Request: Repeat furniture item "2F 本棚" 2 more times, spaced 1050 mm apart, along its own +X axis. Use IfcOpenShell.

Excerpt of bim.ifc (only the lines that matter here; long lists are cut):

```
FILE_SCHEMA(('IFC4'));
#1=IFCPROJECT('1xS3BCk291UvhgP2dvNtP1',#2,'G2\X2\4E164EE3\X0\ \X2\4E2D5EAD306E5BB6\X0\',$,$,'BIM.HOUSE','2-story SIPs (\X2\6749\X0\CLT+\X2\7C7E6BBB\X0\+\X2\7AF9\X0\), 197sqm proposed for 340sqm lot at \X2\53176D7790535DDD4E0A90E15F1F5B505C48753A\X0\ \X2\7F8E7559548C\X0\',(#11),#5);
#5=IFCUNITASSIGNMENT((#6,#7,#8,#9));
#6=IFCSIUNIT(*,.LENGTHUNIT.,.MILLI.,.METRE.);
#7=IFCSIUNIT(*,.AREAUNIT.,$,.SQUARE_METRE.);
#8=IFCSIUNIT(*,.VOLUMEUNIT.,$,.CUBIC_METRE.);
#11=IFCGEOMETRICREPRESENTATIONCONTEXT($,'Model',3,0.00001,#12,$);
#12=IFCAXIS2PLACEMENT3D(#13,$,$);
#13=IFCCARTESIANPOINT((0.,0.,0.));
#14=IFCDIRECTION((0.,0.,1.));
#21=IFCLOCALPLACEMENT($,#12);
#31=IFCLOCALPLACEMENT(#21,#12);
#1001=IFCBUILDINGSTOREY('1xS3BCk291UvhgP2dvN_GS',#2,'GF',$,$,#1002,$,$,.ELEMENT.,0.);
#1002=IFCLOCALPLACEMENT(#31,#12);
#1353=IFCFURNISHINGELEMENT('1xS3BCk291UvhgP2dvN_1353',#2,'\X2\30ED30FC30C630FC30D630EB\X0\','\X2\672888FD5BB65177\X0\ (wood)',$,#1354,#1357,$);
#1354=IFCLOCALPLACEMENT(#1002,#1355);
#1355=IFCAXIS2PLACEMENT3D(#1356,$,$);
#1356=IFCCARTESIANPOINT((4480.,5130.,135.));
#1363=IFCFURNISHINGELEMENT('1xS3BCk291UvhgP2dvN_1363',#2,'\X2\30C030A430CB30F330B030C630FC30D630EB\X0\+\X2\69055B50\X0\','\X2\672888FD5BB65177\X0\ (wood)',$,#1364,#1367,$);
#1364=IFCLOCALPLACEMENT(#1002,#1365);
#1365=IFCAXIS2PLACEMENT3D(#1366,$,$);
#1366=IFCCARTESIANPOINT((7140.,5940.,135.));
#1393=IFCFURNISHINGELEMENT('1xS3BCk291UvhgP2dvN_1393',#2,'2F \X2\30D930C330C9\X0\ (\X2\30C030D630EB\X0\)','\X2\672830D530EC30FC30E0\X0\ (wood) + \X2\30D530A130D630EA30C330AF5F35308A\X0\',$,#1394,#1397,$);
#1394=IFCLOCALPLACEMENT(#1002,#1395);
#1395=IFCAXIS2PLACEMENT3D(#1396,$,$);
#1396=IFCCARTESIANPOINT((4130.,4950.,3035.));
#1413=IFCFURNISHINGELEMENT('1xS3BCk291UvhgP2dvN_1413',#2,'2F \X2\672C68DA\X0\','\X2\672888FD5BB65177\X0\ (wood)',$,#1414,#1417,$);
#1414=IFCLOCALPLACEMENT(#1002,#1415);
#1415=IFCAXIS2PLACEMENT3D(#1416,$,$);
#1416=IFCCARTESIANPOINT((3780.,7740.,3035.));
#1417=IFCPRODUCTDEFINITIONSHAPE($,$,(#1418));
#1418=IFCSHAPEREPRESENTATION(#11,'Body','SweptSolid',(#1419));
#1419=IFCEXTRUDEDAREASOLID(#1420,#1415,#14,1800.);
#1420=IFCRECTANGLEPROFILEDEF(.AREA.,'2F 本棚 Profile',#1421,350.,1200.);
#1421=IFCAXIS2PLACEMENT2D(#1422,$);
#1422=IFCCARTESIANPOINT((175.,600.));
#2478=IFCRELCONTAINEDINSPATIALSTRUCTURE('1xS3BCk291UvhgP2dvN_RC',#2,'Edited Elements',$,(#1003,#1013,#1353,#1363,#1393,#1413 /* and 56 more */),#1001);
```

```python
import ifcopenshell
import ifcopenshell.api.geometry
import ifcopenshell.api.root
import ifcopenshell.util.element
import ifcopenshell.util.placement

model = ifcopenshell.open("bim.ifc")


def reuse_history(source, copy):
    """copy_class also copies each property set's owner history, people and application; keep the originals."""
    for rel in copy.IsDefinedBy:
        if rel.is_a("IfcRelDefinesByProperties") and (history := rel.RelatingPropertyDefinition.OwnerHistory):
            rel.RelatingPropertyDefinition.OwnerHistory = source.OwnerHistory
            ifcopenshell.util.element.remove_deep2(model, history)


source = model.by_id(1413)
base = ifcopenshell.util.placement.get_local_placement(source.ObjectPlacement)
step = base[:3, 0] * 1050.0

for i in range(1, 3):
    copy = ifcopenshell.api.root.copy_class(model, product=source)
    copy.Representation = ifcopenshell.util.element.copy_deep(
        model, source.Representation, exclude=["IfcGeometricRepresentationContext", "IfcRepresentationMap"]
    )
    reuse_history(source, copy)
    matrix = base.copy()
    matrix[:3, 3] += i * step
    print("added at", matrix[:3, 3].round(3) + 0.0)
    ifcopenshell.api.geometry.edit_object_placement(model, product=copy, matrix=matrix, is_si=False)

model.write("bim-out.ifc")
```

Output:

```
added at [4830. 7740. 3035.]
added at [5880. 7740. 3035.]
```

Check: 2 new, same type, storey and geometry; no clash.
